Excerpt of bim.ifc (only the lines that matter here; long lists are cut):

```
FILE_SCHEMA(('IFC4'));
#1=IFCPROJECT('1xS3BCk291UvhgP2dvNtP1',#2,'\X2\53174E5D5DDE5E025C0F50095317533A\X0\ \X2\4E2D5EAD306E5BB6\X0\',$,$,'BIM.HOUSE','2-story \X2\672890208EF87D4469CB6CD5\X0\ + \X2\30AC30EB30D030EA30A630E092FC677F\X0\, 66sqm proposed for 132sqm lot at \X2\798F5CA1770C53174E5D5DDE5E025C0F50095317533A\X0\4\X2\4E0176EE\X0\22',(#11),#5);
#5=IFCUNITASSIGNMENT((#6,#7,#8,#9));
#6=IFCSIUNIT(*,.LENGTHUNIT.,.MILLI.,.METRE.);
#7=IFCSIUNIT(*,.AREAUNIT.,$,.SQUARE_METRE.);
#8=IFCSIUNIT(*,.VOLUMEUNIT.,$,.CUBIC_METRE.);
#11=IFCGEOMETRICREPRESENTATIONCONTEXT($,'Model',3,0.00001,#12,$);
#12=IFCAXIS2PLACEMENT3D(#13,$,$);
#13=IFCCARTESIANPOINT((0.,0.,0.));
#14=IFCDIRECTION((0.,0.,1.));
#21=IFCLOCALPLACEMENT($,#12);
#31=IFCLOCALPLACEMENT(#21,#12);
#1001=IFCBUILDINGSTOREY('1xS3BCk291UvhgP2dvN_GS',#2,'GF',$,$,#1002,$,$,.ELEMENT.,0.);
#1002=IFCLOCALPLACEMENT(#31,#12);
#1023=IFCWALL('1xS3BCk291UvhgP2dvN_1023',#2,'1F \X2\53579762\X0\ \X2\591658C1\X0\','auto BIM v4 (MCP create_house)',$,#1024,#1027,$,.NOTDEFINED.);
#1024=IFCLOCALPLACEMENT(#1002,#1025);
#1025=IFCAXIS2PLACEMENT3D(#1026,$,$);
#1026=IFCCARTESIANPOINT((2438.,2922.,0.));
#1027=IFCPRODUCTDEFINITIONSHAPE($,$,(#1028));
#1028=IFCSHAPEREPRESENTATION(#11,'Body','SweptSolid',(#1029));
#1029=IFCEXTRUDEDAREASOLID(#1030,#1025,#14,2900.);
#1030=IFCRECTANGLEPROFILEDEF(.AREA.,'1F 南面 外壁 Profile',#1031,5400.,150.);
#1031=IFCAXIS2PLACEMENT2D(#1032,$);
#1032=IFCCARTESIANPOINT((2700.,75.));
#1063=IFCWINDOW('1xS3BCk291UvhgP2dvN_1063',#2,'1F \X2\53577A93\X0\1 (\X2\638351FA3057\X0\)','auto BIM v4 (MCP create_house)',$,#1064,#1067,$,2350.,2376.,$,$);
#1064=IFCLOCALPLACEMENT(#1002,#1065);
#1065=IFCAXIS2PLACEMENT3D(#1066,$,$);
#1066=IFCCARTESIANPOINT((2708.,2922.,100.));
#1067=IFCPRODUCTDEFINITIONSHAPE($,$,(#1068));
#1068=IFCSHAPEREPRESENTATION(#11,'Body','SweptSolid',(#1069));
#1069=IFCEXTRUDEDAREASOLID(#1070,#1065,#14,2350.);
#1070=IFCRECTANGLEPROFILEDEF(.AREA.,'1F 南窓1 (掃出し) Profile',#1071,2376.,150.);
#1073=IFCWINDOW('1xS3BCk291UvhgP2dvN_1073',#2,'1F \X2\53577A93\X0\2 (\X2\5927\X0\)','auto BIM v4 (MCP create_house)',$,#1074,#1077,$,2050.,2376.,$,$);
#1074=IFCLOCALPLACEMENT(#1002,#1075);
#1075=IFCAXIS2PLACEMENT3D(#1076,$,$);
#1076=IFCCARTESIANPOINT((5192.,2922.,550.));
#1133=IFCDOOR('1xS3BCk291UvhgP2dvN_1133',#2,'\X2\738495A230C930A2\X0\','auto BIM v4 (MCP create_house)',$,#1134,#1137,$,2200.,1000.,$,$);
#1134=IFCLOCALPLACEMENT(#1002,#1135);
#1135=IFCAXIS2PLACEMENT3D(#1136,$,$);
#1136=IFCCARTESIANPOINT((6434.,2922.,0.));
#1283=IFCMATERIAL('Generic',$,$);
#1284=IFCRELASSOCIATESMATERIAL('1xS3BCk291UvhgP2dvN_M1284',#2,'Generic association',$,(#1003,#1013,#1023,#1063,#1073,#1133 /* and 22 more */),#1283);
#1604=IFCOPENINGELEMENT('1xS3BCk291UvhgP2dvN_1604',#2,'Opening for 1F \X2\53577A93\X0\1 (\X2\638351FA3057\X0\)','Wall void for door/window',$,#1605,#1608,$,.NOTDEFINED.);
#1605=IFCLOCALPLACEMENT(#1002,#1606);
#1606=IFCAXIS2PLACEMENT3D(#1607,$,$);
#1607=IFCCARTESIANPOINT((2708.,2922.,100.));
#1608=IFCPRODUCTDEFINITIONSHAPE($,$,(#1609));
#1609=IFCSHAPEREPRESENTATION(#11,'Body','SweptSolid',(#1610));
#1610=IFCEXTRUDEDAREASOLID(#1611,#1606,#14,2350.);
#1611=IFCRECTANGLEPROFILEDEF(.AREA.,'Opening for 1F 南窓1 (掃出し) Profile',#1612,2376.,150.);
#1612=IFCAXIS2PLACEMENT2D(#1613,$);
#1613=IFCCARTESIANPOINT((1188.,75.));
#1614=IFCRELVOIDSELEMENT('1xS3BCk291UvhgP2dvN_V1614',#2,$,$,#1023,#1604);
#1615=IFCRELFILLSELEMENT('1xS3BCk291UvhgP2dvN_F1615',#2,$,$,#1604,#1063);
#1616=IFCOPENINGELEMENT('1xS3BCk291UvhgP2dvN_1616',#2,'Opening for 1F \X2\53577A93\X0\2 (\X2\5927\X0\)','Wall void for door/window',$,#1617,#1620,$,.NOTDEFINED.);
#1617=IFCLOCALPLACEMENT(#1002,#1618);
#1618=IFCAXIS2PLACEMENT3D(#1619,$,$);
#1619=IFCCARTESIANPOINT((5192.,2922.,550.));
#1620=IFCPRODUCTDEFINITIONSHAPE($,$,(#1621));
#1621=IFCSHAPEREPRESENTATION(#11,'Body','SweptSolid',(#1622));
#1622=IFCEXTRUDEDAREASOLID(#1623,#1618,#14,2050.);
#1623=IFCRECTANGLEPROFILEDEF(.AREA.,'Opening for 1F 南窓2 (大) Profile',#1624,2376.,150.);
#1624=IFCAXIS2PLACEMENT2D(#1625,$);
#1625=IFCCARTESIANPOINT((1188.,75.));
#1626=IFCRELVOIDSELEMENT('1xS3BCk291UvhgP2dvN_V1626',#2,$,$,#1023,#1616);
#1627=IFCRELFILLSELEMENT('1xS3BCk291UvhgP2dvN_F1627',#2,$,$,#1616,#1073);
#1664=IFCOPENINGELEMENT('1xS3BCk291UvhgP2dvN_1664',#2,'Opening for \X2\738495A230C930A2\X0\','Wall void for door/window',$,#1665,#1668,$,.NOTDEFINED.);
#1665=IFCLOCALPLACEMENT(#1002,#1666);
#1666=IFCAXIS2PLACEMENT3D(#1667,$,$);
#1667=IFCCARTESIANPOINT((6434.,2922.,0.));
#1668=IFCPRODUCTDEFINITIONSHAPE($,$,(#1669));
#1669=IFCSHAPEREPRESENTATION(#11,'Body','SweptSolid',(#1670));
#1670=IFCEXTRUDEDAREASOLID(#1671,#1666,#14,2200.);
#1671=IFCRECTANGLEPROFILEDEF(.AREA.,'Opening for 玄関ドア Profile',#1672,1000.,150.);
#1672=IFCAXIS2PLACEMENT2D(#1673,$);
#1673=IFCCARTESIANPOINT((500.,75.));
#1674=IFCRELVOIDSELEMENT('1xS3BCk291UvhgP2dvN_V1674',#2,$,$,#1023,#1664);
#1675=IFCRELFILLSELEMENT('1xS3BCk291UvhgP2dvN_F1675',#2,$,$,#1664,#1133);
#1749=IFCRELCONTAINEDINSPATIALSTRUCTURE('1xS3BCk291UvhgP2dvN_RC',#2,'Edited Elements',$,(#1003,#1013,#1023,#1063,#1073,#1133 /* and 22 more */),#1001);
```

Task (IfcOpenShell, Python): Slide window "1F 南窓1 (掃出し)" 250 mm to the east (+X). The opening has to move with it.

```python
import ifcopenshell
import ifcopenshell.api.geometry
import ifcopenshell.util.placement

model = ifcopenshell.open("bim.ifc")

window = model.by_guid("1xS3BCk291UvhgP2dvN_1063")
opening = window.FillsVoids[0].RelatingOpeningElement
wall = opening.VoidsElements[0].RelatingBuildingElement

wall_matrix = ifcopenshell.util.placement.get_local_placement(wall.ObjectPlacement)
shift = wall_matrix[:3, 0] * 250.0
before = ifcopenshell.util.placement.get_local_placement(window.ObjectPlacement)[:3, 3].copy()

# The window is not placed relative to its opening, so move both.
for product in (opening, window):
    matrix = ifcopenshell.util.placement.get_local_placement(product.ObjectPlacement)
    matrix[:3, 3] += shift
    ifcopenshell.api.geometry.edit_object_placement(model, product=product, matrix=matrix, is_si=False)

after = ifcopenshell.util.placement.get_local_placement(window.ObjectPlacement)[:3, 3]
print("window moved by", (after - before).round(3) + 0.0)

model.write("bim_v2.ifc")
```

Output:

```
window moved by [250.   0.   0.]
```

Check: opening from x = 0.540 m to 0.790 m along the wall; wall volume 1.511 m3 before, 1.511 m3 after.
